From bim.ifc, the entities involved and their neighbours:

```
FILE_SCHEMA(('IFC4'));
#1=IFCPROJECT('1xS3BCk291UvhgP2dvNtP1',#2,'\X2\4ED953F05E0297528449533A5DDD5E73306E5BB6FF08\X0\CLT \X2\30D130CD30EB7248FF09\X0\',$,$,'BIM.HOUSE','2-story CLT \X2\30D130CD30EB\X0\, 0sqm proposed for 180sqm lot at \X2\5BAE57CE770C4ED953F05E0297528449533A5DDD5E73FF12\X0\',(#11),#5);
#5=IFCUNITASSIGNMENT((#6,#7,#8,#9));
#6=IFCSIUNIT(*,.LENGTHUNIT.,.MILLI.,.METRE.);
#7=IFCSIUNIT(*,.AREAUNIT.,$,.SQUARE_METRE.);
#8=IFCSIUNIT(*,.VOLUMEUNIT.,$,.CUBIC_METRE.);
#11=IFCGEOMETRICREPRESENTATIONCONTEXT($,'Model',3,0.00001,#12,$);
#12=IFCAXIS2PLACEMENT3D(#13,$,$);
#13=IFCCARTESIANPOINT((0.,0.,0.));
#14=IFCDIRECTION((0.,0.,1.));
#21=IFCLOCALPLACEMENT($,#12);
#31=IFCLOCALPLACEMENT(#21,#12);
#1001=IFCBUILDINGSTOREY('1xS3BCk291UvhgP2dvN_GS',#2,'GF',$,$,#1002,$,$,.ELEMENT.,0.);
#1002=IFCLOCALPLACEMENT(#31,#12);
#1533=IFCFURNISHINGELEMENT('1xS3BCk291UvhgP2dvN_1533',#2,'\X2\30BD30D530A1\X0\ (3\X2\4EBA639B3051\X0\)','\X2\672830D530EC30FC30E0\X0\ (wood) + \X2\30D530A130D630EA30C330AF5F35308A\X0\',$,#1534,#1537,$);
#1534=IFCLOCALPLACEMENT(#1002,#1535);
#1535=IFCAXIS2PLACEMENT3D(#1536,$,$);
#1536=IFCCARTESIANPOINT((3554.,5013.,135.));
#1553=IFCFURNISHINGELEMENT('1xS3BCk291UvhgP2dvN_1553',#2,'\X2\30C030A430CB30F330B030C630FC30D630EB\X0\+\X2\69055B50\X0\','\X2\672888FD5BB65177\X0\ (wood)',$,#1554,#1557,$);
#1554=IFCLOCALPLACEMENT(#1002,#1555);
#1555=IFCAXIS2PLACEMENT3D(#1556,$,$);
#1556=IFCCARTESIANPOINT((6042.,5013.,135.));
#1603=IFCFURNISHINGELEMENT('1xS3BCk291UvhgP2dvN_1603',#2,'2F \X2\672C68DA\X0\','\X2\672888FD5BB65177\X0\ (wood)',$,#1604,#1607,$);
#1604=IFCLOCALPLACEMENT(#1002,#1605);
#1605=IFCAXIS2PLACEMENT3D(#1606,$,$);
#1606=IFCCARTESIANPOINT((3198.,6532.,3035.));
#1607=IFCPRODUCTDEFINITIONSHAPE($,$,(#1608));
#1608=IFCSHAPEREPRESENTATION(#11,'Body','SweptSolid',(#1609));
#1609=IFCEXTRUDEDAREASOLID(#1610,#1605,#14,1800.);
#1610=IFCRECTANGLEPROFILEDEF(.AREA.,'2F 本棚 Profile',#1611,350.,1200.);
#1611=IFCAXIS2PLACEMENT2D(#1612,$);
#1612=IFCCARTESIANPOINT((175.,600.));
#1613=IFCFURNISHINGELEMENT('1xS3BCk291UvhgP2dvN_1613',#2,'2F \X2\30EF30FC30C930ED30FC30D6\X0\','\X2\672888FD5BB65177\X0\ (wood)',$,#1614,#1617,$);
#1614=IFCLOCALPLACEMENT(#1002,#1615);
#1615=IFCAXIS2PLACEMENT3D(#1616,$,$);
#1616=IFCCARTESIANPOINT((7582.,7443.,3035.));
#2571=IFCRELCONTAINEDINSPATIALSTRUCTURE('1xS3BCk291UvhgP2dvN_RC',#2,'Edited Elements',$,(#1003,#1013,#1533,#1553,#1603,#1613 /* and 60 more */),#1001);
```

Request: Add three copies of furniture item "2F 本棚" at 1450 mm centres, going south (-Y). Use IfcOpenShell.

```python
import numpy as np
import ifcopenshell
import ifcopenshell.api.geometry
import ifcopenshell.api.root
import ifcopenshell.util.element
import ifcopenshell.util.placement

model = ifcopenshell.open("bim.ifc")


def reuse_history(source, copy):
    """copy_class also copies each property set's owner history, people and application; keep the originals."""
    for rel in copy.IsDefinedBy:
        if rel.is_a("IfcRelDefinesByProperties") and (history := rel.RelatingPropertyDefinition.OwnerHistory):
            rel.RelatingPropertyDefinition.OwnerHistory = source.OwnerHistory
            ifcopenshell.util.element.remove_deep2(model, history)


source = model.by_guid("1xS3BCk291UvhgP2dvN_1603")
base = ifcopenshell.util.placement.get_local_placement(source.ObjectPlacement)
step = np.array([0.0, -1.0, 0.0]) * 1450.0

for i in range(1, 4):
    copy = ifcopenshell.api.root.copy_class(model, product=source)
    copy.Representation = ifcopenshell.util.element.copy_deep(
        model, source.Representation, exclude=["IfcGeometricRepresentationContext", "IfcRepresentationMap"]
    )
    reuse_history(source, copy)
    matrix = base.copy()
    matrix[:3, 3] += i * step
    print("added at", matrix[:3, 3].round(3) + 0.0)
    ifcopenshell.api.geometry.edit_object_placement(model, product=copy, matrix=matrix, is_si=False)

model.write("bim-out.ifc")
```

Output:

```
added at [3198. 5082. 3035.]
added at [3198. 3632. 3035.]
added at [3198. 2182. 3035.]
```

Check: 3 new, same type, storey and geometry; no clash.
